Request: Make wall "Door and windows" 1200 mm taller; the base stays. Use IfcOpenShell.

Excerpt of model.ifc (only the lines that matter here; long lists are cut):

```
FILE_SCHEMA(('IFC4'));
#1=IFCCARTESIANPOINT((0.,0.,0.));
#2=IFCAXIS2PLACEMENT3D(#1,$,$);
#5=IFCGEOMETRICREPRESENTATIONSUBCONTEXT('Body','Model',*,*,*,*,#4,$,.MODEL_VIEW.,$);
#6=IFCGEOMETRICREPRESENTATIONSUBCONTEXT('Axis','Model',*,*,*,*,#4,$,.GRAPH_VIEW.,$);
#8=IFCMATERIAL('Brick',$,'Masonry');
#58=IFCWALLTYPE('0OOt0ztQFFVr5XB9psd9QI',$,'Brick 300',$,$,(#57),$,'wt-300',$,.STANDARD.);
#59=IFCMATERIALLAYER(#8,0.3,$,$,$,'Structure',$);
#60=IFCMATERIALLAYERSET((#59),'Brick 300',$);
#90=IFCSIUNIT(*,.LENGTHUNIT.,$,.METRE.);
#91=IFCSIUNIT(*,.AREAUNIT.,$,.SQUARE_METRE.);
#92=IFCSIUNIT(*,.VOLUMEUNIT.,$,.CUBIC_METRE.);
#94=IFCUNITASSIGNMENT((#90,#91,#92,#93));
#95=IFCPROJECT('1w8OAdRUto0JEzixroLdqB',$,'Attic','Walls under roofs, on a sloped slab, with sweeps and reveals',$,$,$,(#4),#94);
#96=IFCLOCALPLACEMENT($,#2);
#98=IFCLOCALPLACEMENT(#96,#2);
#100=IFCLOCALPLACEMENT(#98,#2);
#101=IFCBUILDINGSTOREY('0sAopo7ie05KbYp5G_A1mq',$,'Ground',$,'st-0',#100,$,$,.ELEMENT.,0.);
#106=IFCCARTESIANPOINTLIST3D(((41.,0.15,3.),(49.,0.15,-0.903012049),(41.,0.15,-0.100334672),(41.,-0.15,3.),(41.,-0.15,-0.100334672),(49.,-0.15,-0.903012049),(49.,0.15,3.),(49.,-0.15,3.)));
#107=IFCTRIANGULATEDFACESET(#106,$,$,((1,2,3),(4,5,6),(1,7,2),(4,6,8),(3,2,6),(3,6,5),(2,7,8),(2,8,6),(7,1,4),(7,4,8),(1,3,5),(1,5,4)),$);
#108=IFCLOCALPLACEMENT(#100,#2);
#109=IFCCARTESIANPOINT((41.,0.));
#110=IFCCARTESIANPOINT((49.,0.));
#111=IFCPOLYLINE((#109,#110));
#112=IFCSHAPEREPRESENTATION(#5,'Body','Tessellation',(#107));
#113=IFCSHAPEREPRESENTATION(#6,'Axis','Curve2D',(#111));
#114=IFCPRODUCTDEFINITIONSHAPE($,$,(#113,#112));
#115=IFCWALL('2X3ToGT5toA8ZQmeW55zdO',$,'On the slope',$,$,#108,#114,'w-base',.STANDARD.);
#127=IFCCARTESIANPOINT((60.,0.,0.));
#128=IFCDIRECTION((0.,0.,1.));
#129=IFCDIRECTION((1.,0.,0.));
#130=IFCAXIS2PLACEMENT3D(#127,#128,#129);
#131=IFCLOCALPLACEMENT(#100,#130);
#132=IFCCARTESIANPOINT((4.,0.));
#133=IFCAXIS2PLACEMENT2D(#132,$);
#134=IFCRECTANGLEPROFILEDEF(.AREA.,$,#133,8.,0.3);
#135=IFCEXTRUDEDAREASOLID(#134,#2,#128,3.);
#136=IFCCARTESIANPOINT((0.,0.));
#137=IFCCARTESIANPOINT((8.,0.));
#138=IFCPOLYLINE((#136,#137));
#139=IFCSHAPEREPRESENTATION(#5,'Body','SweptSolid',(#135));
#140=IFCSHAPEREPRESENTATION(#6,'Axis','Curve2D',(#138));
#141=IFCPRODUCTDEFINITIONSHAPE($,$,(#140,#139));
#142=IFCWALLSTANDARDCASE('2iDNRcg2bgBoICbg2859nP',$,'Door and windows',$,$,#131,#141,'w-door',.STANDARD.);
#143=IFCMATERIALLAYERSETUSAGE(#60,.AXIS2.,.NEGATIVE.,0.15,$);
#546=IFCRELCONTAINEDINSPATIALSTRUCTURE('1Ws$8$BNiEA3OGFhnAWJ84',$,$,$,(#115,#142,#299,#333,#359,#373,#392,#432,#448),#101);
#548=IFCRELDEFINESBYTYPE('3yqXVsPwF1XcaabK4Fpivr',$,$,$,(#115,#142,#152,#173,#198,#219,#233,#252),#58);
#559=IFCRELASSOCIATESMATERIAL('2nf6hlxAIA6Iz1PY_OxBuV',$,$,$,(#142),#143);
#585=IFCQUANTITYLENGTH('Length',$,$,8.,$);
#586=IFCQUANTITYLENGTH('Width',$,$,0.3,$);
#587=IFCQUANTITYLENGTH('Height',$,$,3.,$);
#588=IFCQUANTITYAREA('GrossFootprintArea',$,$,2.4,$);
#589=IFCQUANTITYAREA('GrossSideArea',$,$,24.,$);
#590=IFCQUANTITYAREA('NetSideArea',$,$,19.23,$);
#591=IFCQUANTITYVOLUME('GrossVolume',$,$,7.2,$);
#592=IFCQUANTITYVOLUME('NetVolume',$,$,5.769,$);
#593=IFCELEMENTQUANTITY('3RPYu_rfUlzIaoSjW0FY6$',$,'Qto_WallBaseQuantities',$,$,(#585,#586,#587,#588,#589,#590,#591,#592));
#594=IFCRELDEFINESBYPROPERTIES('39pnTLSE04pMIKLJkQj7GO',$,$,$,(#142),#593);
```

```python
import ifcopenshell
import ifcopenshell.api.pset
import ifcopenshell.geom
import ifcopenshell.util.element
import ifcopenshell.util.representation
import ifcopenshell.util.shape
import ifcopenshell.util.unit

model = ifcopenshell.open("model.ifc")
unit_scale = ifcopenshell.util.unit.calculate_unit_scale(model)
area_scale = ifcopenshell.util.unit.calculate_unit_scale(model, "AREAUNIT")
volume_scale = ifcopenshell.util.unit.calculate_unit_scale(model, "VOLUMEUNIT")
settings = ifcopenshell.geom.settings()


def volume(element):
    """Net volume in cubic metres, openings subtracted."""
    shape = ifcopenshell.geom.create_shape(settings, element)
    return ifcopenshell.util.shape.get_volume(shape.geometry)


wall = model.by_guid("2iDNRcg2bgBoICbg2859nP")
before = volume(wall)

body = ifcopenshell.util.representation.get_representation(wall, "Model", "Body")
solid = body.Items[0]
old_height = solid.Depth
solid.Depth += 1.2 / unit_scale
after = volume(wall)
thickness = 0.3  # wall thickness in metres

# Update the stored height, areas and volumes.
qto = model.by_id(ifcopenshell.util.element.get_pset(wall, "Qto_WallBaseQuantities", should_inherit=False)["id"])
ifcopenshell.api.pset.edit_qto(model, qto=qto, properties={
    "Height": solid.Depth,
    "GrossSideArea": ifcopenshell.util.element.get_pset(wall, "Qto_WallBaseQuantities", "GrossSideArea") * solid.Depth / old_height,
    "NetSideArea": after / thickness / area_scale,
    "GrossVolume": ifcopenshell.util.element.get_pset(wall, "Qto_WallBaseQuantities", "GrossVolume") * solid.Depth / old_height,
    "NetVolume": after / volume_scale,
})

print(f"height {old_height:g} -> {solid.Depth:g}, volume {before:.3f} -> {after:.3f} m3")

model.write("model_rev.ifc")
```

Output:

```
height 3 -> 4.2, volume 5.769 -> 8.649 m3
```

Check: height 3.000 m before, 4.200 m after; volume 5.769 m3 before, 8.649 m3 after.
